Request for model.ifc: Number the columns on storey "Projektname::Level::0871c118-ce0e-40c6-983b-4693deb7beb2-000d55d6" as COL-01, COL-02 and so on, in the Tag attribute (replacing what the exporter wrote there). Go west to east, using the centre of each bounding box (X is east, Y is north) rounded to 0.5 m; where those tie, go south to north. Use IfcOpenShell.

First a look at what the model holds.

```python
import ifcopenshell
import ifcopenshell.util.element
import ifcopenshell.util.placement

model = ifcopenshell.open("model.ifc")
print(model.schema)
storey = next(s for s in model.by_type("IfcBuildingStorey") if s.Name == "Projektname::Level::0871c118-ce0e-40c6-983b-4693deb7beb2-000d55d6")
columns = [e for e in ifcopenshell.util.element.get_decomposition(storey) if e.is_a("IfcColumn")]
for e in sorted(columns, key=lambda e: e.id()):
    origin = ifcopenshell.util.placement.get_local_placement(e.ObjectPlacement)[:3, 3]
    print(e.id(), e.Tag, e.Name, origin.round(2) + 0.0, sep=" | ")
```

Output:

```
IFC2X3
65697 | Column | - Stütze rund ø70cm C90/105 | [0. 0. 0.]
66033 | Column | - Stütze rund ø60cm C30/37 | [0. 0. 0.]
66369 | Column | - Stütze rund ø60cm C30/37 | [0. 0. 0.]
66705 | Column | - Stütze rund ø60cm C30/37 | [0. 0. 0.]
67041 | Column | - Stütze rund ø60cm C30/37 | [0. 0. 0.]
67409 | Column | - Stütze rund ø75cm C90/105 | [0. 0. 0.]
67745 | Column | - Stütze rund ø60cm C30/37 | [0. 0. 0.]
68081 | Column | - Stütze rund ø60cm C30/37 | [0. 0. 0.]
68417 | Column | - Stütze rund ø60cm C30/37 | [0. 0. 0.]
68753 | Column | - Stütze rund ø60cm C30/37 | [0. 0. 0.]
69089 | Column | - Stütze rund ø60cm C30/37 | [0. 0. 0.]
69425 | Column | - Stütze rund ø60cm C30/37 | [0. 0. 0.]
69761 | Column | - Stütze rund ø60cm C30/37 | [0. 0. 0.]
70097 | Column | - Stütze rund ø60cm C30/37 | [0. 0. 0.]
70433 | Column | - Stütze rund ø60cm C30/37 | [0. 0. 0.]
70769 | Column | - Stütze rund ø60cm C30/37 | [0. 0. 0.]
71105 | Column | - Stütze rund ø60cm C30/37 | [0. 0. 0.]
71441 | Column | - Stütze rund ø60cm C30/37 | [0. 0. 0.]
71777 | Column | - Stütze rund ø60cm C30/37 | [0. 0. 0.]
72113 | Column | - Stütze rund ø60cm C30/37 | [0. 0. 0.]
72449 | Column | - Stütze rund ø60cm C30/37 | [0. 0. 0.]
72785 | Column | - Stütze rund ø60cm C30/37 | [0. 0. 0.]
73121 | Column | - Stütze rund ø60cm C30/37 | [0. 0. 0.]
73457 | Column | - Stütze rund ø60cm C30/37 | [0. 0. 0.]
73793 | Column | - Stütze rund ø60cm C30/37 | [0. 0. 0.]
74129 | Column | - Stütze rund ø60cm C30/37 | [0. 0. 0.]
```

```python
import ifcopenshell
import ifcopenshell.geom
import ifcopenshell.util.element
import ifcopenshell.util.shape

model = ifcopenshell.open("model.ifc")
settings = ifcopenshell.geom.settings()
settings.set("use-world-coords", True)


def centre(element):
    shape = ifcopenshell.geom.create_shape(settings, element)
    return ifcopenshell.util.shape.get_bbox_centroid(shape.geometry)


storey = next(s for s in model.by_type("IfcBuildingStorey") if s.Name == "Projektname::Level::0871c118-ce0e-40c6-983b-4693deb7beb2-000d55d6")
columns = [e for e in ifcopenshell.util.element.get_decomposition(storey) if e.is_a("IfcColumn")]

# Insertion points can sit at a corner or the storey origin, so sort by the geometry (in metres).
centres = {e: centre(e) for e in columns}
columns.sort(key=lambda e: (round(centres[e][0] / 0.5), centres[e][1]))

for i, e in enumerate(columns, start=1):
    number = f"COL-{i:02d}"
    e.Tag = number
    print(e.id(), number)

model.write("model_v2.ifc")
```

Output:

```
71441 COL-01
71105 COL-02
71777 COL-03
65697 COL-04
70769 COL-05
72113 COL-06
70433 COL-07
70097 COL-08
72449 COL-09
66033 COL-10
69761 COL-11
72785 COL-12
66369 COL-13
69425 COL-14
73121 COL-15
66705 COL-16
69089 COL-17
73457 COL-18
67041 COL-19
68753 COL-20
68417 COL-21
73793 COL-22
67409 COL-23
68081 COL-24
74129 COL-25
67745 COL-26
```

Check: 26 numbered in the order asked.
